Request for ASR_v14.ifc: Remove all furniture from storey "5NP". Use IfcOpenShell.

First a look at what the model holds.

```python
import ifcopenshell
import ifcopenshell.util.element

model = ifcopenshell.open("ASR_v14.ifc")
print(model.schema)
storey = next(s for s in model.by_type("IfcBuildingStorey") if s.Name == "5NP")
furniture = [e for e in ifcopenshell.util.element.get_decomposition(storey) if e.is_a("IfcFurnishingElement")]
seen = {}
for e in furniture:
    element_type = ifcopenshell.util.element.get_type(e)
    name = element_type.Name if element_type not in (None, e) else None
    seen[name] = seen.get(name, 0) + 1
for name, count in sorted(seen.items(), key=str):
    print(count, "x", name)
```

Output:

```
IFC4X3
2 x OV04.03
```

```python
import ifcopenshell
import ifcopenshell.api.root
import ifcopenshell.util.element

model = ifcopenshell.open("ASR_v14.ifc")

storey = next(s for s in model.by_type("IfcBuildingStorey") if s.Name == "5NP")
furniture = [e for e in ifcopenshell.util.element.get_decomposition(storey) if e.is_a("IfcFurnishingElement")]

for e in furniture:
    ifcopenshell.api.root.remove_product(model, product=e)
print(len(furniture), "removed")

model.write("ASR_v14_rev.ifc")
```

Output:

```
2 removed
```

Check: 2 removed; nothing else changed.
